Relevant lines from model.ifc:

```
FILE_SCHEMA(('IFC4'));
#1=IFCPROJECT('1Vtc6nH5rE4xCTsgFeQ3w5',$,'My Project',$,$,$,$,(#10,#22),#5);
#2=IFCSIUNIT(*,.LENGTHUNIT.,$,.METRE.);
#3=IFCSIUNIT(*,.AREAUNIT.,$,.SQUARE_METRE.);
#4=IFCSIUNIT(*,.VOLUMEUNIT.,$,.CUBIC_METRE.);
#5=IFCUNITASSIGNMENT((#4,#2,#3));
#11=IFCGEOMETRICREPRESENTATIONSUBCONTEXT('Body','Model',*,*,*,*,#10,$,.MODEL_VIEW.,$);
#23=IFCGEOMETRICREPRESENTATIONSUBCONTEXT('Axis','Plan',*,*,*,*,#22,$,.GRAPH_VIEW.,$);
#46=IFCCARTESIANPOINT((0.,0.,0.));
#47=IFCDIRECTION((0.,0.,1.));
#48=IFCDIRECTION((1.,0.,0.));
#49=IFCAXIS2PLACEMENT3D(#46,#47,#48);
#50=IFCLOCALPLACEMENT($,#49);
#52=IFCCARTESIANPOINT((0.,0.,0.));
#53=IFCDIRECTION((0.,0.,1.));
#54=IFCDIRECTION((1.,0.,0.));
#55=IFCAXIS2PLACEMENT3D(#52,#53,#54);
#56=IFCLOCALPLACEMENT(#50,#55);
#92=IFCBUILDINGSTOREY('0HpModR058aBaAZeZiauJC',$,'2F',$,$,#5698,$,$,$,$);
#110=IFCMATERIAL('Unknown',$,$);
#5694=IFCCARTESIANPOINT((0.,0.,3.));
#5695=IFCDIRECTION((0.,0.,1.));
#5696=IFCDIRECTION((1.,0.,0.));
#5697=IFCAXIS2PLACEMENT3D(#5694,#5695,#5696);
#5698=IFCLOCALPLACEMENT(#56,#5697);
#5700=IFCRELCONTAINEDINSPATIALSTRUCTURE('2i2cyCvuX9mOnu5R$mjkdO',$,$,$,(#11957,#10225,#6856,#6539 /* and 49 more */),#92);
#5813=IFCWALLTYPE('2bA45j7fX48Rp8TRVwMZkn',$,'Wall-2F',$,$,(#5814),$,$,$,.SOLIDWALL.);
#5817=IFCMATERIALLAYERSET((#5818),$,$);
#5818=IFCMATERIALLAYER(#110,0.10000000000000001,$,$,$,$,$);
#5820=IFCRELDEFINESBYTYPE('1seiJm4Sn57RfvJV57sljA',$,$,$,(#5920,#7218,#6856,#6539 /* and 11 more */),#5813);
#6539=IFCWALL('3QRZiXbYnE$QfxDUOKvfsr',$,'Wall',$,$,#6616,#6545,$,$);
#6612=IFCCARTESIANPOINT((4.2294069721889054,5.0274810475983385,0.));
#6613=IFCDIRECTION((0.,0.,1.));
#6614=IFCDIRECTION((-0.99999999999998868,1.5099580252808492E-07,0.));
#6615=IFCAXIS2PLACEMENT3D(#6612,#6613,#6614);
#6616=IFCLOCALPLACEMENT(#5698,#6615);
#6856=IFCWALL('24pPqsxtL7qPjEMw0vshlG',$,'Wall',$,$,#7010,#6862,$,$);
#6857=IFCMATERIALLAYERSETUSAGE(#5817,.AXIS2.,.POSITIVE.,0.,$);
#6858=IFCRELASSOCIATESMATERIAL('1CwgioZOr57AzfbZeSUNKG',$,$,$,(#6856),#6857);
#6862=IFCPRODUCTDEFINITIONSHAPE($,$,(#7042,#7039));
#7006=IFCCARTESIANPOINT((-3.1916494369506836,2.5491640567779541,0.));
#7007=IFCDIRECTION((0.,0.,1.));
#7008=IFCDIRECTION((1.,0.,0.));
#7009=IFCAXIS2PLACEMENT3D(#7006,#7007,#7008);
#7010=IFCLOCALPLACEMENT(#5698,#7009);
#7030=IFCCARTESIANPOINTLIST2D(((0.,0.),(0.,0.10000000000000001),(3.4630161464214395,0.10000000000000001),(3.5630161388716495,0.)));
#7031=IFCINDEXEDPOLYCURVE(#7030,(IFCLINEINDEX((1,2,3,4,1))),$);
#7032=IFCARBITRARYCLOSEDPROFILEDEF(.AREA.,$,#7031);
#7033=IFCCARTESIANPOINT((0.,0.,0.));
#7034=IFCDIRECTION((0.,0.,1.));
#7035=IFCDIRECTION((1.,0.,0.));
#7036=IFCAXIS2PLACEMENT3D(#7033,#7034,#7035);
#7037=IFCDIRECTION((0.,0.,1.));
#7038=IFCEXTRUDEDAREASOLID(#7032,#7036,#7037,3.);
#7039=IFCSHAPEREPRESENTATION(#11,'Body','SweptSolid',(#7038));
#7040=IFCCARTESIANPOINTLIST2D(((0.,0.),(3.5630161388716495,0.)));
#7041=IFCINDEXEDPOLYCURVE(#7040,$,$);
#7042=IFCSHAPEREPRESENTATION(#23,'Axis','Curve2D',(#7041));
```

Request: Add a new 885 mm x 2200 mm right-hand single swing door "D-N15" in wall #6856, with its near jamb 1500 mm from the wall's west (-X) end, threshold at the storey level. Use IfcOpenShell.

```python
import numpy as np
import ifcopenshell
import ifcopenshell.api.feature
import ifcopenshell.api.geometry
import ifcopenshell.api.root
import ifcopenshell.api.spatial
import ifcopenshell.geom
import ifcopenshell.util.element
import ifcopenshell.util.placement
import ifcopenshell.util.representation
import ifcopenshell.util.shape
import ifcopenshell.util.unit

model = ifcopenshell.open("model.ifc")
unit_scale = ifcopenshell.util.unit.calculate_unit_scale(model)
settings = ifcopenshell.geom.settings()


def volume(element):
    """Net volume in cubic metres, openings subtracted."""
    shape = ifcopenshell.geom.create_shape(settings, element)
    return ifcopenshell.util.shape.get_volume(shape.geometry)


wall = model.by_id(6856)
storey = ifcopenshell.util.element.get_container(wall, ifc_class="IfcBuildingStorey")
context = ifcopenshell.util.representation.get_context(model, "Model", "Body", "MODEL_VIEW")
before = volume(wall)

width, height, from_end, sill = 0.885, 2.2, 1.5, 0.0  # metres

# The wall runs along its own X axis, and the end named is its -X end.
wall_shape = ifcopenshell.geom.create_shape(settings, wall)
x, y, z = ifcopenshell.util.shape.get_vertices(wall_shape.geometry).T
start = x.min() + from_end
face, thickness = float(y.min()), float(y.max() - y.min())
wall_matrix = ifcopenshell.util.placement.get_local_placement(wall.ObjectPlacement)
level = ifcopenshell.util.placement.get_local_placement(storey.ObjectPlacement)[2, 3]


def in_wall(x, y):
    """Placement at x, y metres in the wall's axes, at sill height."""
    matrix = wall_matrix.copy()
    matrix[:, 3] = wall_matrix @ np.array([x / unit_scale, y / unit_scale, 0.0, 1.0])
    matrix[2, 3] = level + sill / unit_scale
    return matrix


# Opening: a box that overshoots both wall faces by 50 mm.
opening = ifcopenshell.api.root.create_entity(model, ifc_class="IfcOpeningElement", predefined_type="OPENING")
box = ifcopenshell.api.geometry.add_wall_representation(
    model, context=context, length=width, height=height, thickness=thickness + 0.1
)
ifcopenshell.api.geometry.assign_representation(model, product=opening, representation=box)
ifcopenshell.api.geometry.edit_object_placement(model, product=opening, matrix=in_wall(start, face - 0.05), is_si=False)
ifcopenshell.api.feature.add_feature(model, feature=opening, element=wall)

door = ifcopenshell.api.root.create_entity(model, ifc_class="IfcDoor", name="D-N15", predefined_type="DOOR")
door.OverallWidth, door.OverallHeight = width / unit_scale, height / unit_scale
door.OperationType = "SINGLE_SWING_RIGHT"
body = ifcopenshell.api.geometry.add_door_representation(
    model,
    context=context,
    overall_width=door.OverallWidth,
    overall_height=door.OverallHeight,
    operation_type="SINGLE_SWING_RIGHT",
    lining_properties={"LiningDepth": thickness / unit_scale, "ThresholdDepth": thickness / unit_scale},
)
ifcopenshell.api.geometry.assign_representation(model, product=door, representation=body)
ifcopenshell.api.spatial.assign_container(model, products=[door], relating_structure=storey)
ifcopenshell.api.feature.add_filling(model, opening=opening, element=door)

# The lining spans the wall, so the door starts at the wall face.
ifcopenshell.api.geometry.edit_object_placement(model, product=door, matrix=in_wall(start, face), is_si=False)

after = volume(wall)

print(f"wall volume {before:.3f} -> {after:.3f} m3")

model.write("model_v2.ifc")
```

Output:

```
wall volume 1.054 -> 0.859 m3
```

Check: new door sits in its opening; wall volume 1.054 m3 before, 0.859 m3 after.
